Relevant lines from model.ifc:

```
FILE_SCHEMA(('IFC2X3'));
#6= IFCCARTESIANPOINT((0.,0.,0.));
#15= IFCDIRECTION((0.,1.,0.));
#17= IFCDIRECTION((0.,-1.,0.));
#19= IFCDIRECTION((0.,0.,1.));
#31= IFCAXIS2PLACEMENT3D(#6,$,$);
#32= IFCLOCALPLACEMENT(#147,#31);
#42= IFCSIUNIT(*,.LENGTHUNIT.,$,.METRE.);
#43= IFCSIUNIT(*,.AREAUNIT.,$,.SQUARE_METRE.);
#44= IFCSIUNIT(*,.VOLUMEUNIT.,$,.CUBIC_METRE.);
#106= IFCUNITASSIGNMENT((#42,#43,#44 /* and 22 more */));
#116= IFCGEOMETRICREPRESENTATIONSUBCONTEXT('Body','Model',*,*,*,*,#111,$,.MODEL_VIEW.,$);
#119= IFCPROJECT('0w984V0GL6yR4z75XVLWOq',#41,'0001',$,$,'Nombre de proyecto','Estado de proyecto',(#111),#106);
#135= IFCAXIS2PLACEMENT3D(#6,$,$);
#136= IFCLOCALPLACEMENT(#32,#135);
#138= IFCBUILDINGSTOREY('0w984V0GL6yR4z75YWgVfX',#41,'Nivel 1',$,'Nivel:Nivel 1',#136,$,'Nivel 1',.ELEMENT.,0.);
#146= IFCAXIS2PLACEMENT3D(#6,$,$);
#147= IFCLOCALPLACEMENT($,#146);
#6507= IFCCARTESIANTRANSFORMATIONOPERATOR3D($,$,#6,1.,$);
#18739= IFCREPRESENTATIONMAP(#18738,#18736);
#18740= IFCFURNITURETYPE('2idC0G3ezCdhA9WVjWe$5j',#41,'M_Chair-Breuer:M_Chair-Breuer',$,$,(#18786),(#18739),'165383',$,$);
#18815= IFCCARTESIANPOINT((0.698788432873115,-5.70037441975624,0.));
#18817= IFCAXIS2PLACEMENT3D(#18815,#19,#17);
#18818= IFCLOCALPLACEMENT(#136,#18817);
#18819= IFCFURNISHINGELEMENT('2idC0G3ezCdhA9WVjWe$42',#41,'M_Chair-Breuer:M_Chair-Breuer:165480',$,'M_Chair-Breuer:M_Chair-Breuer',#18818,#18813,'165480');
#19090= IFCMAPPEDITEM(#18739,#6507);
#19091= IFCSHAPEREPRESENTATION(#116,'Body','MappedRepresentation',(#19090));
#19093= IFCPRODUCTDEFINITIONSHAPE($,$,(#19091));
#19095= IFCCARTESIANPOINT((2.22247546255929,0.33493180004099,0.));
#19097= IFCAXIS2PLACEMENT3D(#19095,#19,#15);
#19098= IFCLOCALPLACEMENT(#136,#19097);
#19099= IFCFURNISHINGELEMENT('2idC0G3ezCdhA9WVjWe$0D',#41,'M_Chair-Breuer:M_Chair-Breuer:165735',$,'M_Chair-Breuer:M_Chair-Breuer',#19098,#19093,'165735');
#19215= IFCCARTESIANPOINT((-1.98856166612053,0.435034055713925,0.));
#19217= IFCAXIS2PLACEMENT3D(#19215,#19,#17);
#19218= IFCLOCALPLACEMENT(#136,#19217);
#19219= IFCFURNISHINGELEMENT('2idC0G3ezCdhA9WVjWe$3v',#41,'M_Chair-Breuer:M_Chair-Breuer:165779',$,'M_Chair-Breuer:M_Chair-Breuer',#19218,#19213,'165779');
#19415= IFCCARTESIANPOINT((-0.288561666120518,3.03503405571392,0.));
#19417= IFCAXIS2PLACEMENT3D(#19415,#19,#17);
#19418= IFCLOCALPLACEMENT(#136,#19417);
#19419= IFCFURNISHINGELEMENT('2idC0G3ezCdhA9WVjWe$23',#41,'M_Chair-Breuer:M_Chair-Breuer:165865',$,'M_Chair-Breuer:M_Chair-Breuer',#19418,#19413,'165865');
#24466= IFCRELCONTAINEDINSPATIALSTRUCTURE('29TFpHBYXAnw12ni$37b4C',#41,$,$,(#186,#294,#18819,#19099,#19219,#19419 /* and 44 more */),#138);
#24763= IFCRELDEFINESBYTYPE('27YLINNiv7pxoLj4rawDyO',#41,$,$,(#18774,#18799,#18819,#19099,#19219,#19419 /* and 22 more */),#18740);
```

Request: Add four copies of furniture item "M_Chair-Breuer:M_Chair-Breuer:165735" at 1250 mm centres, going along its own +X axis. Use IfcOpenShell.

```python
import ifcopenshell
import ifcopenshell.api.geometry
import ifcopenshell.api.root
import ifcopenshell.util.element
import ifcopenshell.util.placement
import ifcopenshell.util.unit

model = ifcopenshell.open("model.ifc")
unit_scale = ifcopenshell.util.unit.calculate_unit_scale(model)


def reuse_history(source, copy):
    """copy_class also copies each property set's owner history, people and application; keep the originals."""
    for rel in copy.IsDefinedBy:
        if rel.is_a("IfcRelDefinesByProperties") and (history := rel.RelatingPropertyDefinition.OwnerHistory):
            rel.RelatingPropertyDefinition.OwnerHistory = source.OwnerHistory
            ifcopenshell.util.element.remove_deep2(model, history)


source = model.by_guid("2idC0G3ezCdhA9WVjWe$0D")
base = ifcopenshell.util.placement.get_local_placement(source.ObjectPlacement)
step = base[:3, 0] * 1.25 / unit_scale

for i in range(1, 5):
    copy = ifcopenshell.api.root.copy_class(model, product=source)
    copy.Representation = ifcopenshell.util.element.copy_deep(
        model, source.Representation, exclude=["IfcGeometricRepresentationContext", "IfcRepresentationMap"]
    )
    copy.Name = "M_Chair-Breuer:M_Chair-Breuer"
    copy.Tag = None
    reuse_history(source, copy)
    matrix = base.copy()
    matrix[:3, 3] += i * step
    print("added at", matrix[:3, 3].round(3) + 0.0)
    ifcopenshell.api.geometry.edit_object_placement(model, product=copy, matrix=matrix, is_si=False)

model.write("model_edited.ifc")
```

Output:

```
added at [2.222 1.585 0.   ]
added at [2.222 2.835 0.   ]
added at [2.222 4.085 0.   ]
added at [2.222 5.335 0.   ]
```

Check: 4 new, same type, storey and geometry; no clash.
